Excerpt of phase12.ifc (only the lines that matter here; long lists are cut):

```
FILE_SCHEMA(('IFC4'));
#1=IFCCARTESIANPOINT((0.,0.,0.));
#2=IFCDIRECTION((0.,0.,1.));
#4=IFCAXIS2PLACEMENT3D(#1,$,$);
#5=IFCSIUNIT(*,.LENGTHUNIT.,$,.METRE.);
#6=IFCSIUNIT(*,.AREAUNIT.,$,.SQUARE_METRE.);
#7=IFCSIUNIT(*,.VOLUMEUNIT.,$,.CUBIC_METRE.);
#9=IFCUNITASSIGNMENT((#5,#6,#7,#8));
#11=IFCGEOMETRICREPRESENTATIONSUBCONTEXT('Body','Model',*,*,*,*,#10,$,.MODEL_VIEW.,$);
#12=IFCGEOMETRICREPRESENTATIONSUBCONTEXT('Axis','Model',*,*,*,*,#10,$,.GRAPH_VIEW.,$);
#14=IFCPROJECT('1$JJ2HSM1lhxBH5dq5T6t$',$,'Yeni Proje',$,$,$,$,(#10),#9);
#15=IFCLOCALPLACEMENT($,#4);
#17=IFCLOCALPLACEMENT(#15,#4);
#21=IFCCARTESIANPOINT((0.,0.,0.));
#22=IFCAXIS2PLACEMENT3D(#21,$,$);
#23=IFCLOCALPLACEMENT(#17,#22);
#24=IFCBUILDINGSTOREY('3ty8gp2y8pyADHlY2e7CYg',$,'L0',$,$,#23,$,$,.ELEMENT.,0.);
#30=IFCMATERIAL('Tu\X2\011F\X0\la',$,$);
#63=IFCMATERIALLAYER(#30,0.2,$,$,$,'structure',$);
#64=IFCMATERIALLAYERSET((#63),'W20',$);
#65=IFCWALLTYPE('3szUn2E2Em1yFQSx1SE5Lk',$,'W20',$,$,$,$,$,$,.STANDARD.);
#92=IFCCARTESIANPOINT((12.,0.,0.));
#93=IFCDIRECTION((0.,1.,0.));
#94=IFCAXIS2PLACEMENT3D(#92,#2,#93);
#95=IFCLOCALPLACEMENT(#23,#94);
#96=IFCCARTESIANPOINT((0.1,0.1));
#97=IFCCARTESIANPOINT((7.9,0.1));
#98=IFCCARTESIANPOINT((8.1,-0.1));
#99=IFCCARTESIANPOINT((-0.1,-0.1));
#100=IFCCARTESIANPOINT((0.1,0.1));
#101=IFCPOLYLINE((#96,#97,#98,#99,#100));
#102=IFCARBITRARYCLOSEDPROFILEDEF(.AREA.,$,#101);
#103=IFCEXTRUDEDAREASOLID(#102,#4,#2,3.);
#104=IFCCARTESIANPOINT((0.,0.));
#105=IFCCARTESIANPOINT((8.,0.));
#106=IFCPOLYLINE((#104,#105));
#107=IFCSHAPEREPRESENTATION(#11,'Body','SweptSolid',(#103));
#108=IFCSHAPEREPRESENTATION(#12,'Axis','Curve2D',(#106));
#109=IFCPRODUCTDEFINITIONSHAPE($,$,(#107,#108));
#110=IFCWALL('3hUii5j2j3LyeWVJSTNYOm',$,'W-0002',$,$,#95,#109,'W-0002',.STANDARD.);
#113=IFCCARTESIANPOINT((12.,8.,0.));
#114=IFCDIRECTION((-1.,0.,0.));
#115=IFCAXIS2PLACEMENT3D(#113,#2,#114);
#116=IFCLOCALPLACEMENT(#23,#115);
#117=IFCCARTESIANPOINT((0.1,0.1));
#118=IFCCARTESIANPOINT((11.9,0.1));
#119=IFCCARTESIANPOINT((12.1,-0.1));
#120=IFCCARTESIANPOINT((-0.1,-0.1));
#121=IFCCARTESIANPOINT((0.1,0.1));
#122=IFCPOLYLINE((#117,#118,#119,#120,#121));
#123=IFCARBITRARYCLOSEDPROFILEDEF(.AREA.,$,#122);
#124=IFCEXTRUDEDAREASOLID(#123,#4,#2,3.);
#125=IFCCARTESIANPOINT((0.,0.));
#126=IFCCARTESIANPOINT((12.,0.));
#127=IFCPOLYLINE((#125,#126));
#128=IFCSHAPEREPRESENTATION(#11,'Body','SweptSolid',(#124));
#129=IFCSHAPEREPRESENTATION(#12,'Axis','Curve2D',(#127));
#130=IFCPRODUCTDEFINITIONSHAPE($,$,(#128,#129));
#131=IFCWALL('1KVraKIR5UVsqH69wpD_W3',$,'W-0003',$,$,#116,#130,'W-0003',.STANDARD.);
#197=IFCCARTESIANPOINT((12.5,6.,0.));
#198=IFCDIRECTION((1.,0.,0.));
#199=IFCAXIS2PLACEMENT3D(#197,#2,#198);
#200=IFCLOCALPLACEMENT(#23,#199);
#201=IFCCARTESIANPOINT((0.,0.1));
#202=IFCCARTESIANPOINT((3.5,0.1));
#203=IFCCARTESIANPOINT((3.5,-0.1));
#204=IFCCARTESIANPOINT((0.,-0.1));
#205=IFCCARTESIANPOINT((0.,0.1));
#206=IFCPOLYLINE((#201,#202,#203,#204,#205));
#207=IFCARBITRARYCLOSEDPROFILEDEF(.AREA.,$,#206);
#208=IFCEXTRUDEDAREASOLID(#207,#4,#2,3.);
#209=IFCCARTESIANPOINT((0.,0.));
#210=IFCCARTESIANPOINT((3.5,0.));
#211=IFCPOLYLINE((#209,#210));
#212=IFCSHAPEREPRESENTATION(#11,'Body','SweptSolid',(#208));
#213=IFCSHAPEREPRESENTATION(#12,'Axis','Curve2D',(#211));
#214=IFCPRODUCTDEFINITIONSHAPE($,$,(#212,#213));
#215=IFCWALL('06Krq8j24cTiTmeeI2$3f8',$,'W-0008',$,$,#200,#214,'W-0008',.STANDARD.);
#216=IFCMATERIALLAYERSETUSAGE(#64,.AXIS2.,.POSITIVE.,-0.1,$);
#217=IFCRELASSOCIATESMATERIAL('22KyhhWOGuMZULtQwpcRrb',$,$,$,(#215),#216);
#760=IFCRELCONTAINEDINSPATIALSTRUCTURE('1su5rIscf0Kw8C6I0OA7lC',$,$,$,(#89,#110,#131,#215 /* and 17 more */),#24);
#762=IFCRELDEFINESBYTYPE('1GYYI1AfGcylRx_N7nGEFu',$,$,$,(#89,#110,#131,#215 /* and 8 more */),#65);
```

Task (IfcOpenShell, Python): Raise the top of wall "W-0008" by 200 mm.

```python
import ifcopenshell
import ifcopenshell.geom
import ifcopenshell.util.representation
import ifcopenshell.util.shape

model = ifcopenshell.open("phase12.ifc")
settings = ifcopenshell.geom.settings()


def volume(element):
    """Net volume in cubic metres, openings subtracted."""
    shape = ifcopenshell.geom.create_shape(settings, element)
    return ifcopenshell.util.shape.get_volume(shape.geometry)


wall = model.by_id(215)
before = volume(wall)

body = ifcopenshell.util.representation.get_representation(wall, "Model", "Body")
solid = body.Items[0]
old_height = solid.Depth
solid.Depth += 0.2
after = volume(wall)

print(f"height {old_height:g} -> {solid.Depth:g}, volume {before:.3f} -> {after:.3f} m3")

model.write("phase12_updated.ifc")
```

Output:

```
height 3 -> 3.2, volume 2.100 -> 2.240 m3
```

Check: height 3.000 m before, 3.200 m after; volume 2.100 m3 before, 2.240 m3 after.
